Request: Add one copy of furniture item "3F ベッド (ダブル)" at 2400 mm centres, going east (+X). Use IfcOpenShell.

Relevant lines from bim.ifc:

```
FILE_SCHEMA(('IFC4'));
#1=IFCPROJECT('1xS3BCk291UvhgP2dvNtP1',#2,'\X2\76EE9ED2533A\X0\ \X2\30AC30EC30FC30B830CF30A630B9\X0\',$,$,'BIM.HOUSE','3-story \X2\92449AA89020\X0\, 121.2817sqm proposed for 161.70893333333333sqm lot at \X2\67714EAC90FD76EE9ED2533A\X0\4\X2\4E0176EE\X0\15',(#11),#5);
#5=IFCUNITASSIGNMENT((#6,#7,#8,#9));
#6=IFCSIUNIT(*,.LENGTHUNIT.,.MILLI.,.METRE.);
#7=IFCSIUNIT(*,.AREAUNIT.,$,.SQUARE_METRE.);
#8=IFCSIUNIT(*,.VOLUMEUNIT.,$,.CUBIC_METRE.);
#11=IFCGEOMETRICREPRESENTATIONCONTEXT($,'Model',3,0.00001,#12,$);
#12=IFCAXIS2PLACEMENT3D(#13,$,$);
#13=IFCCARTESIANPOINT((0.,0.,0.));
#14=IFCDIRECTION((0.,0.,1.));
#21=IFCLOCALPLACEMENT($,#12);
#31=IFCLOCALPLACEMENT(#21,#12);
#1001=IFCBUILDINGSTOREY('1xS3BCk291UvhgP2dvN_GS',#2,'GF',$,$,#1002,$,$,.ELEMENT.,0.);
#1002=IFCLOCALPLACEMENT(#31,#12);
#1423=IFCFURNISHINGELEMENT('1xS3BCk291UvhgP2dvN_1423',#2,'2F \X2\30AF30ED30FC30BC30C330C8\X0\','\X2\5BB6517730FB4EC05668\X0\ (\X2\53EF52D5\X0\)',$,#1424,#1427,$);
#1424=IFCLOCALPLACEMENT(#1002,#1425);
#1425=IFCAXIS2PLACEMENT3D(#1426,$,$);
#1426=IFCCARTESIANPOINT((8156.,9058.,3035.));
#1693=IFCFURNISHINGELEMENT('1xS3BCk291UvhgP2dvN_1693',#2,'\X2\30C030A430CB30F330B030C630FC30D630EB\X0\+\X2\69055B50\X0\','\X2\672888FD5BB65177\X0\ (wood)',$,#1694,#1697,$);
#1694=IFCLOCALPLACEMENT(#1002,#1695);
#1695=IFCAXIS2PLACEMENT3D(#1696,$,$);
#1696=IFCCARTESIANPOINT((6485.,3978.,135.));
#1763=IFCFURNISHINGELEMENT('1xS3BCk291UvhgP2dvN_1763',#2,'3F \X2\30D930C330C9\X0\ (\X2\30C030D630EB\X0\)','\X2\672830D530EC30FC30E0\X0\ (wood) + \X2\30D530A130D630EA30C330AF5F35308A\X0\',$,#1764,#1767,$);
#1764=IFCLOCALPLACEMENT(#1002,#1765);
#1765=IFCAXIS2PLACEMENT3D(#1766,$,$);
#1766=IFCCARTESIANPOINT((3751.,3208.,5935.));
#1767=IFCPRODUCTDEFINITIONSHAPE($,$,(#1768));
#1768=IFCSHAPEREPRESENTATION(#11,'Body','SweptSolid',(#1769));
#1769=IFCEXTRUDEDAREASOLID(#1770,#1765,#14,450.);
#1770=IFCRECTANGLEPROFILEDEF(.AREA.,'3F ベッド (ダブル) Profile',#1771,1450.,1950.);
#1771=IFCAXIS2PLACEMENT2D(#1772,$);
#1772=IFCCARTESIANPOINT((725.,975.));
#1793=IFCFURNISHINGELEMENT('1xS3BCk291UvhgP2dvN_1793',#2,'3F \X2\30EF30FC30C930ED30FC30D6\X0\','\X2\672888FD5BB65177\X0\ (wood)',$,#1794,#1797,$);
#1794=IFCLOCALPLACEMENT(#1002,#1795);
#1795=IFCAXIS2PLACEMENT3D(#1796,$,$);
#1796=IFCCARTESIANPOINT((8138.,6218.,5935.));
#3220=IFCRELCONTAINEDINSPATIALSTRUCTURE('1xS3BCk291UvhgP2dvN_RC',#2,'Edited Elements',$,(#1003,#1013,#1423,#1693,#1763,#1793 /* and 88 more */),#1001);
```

```python
import numpy as np
import ifcopenshell
import ifcopenshell.api.geometry
import ifcopenshell.api.root
import ifcopenshell.util.element
import ifcopenshell.util.placement

model = ifcopenshell.open("bim.ifc")


def reuse_history(source, copy):
    """copy_class also copies each property set's owner history, people and application; keep the originals."""
    for rel in copy.IsDefinedBy:
        if rel.is_a("IfcRelDefinesByProperties") and (history := rel.RelatingPropertyDefinition.OwnerHistory):
            rel.RelatingPropertyDefinition.OwnerHistory = source.OwnerHistory
            ifcopenshell.util.element.remove_deep2(model, history)


source = model.by_guid("1xS3BCk291UvhgP2dvN_1763")
base = ifcopenshell.util.placement.get_local_placement(source.ObjectPlacement)
step = np.array([1.0, 0.0, 0.0]) * 2400.0

for i in range(1, 2):
    copy = ifcopenshell.api.root.copy_class(model, product=source)
    copy.Representation = ifcopenshell.util.element.copy_deep(
        model, source.Representation, exclude=["IfcGeometricRepresentationContext", "IfcRepresentationMap"]
    )
    reuse_history(source, copy)
    matrix = base.copy()
    matrix[:3, 3] += i * step
    print("added at", matrix[:3, 3].round(3) + 0.0)
    ifcopenshell.api.geometry.edit_object_placement(model, product=copy, matrix=matrix, is_si=False)

model.write("bim_updated.ifc")
```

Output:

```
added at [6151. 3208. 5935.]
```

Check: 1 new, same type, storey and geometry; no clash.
